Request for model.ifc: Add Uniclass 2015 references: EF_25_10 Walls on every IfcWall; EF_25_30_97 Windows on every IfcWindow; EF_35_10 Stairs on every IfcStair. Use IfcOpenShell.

First a look at what the model holds.

```python
import ifcopenshell

model = ifcopenshell.open("model.ifc")
print(model.schema)
print("classifications:", [c.Name for c in model.by_type("IfcClassification")])
for ifc_class in ("IfcDoor", "IfcRoof", "IfcStair", "IfcWall", "IfcWindow"):
    print(ifc_class, len(model.by_type(ifc_class)))
```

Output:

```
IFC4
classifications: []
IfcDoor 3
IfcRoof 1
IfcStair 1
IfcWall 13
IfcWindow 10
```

```python
import ifcopenshell
import ifcopenshell.api.classification

model = ifcopenshell.open("model.ifc")

system = ifcopenshell.api.classification.add_classification(model, classification="Uniclass 2015")

codes = {
    "IfcWall": ("EF_25_10", "Walls"),
    "IfcWindow": ("EF_25_30_97", "Windows"),
    "IfcStair": ("EF_35_10", "Stairs"),
}
for ifc_class, (code, name) in codes.items():
    products = model.by_type(ifc_class)
    ifcopenshell.api.classification.add_reference(
        model, products=products, classification=system, identification=code, name=name
    )
    print(code, len(products))

model.write("model_updated.ifc")
```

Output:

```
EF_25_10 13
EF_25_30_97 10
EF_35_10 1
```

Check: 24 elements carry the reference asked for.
